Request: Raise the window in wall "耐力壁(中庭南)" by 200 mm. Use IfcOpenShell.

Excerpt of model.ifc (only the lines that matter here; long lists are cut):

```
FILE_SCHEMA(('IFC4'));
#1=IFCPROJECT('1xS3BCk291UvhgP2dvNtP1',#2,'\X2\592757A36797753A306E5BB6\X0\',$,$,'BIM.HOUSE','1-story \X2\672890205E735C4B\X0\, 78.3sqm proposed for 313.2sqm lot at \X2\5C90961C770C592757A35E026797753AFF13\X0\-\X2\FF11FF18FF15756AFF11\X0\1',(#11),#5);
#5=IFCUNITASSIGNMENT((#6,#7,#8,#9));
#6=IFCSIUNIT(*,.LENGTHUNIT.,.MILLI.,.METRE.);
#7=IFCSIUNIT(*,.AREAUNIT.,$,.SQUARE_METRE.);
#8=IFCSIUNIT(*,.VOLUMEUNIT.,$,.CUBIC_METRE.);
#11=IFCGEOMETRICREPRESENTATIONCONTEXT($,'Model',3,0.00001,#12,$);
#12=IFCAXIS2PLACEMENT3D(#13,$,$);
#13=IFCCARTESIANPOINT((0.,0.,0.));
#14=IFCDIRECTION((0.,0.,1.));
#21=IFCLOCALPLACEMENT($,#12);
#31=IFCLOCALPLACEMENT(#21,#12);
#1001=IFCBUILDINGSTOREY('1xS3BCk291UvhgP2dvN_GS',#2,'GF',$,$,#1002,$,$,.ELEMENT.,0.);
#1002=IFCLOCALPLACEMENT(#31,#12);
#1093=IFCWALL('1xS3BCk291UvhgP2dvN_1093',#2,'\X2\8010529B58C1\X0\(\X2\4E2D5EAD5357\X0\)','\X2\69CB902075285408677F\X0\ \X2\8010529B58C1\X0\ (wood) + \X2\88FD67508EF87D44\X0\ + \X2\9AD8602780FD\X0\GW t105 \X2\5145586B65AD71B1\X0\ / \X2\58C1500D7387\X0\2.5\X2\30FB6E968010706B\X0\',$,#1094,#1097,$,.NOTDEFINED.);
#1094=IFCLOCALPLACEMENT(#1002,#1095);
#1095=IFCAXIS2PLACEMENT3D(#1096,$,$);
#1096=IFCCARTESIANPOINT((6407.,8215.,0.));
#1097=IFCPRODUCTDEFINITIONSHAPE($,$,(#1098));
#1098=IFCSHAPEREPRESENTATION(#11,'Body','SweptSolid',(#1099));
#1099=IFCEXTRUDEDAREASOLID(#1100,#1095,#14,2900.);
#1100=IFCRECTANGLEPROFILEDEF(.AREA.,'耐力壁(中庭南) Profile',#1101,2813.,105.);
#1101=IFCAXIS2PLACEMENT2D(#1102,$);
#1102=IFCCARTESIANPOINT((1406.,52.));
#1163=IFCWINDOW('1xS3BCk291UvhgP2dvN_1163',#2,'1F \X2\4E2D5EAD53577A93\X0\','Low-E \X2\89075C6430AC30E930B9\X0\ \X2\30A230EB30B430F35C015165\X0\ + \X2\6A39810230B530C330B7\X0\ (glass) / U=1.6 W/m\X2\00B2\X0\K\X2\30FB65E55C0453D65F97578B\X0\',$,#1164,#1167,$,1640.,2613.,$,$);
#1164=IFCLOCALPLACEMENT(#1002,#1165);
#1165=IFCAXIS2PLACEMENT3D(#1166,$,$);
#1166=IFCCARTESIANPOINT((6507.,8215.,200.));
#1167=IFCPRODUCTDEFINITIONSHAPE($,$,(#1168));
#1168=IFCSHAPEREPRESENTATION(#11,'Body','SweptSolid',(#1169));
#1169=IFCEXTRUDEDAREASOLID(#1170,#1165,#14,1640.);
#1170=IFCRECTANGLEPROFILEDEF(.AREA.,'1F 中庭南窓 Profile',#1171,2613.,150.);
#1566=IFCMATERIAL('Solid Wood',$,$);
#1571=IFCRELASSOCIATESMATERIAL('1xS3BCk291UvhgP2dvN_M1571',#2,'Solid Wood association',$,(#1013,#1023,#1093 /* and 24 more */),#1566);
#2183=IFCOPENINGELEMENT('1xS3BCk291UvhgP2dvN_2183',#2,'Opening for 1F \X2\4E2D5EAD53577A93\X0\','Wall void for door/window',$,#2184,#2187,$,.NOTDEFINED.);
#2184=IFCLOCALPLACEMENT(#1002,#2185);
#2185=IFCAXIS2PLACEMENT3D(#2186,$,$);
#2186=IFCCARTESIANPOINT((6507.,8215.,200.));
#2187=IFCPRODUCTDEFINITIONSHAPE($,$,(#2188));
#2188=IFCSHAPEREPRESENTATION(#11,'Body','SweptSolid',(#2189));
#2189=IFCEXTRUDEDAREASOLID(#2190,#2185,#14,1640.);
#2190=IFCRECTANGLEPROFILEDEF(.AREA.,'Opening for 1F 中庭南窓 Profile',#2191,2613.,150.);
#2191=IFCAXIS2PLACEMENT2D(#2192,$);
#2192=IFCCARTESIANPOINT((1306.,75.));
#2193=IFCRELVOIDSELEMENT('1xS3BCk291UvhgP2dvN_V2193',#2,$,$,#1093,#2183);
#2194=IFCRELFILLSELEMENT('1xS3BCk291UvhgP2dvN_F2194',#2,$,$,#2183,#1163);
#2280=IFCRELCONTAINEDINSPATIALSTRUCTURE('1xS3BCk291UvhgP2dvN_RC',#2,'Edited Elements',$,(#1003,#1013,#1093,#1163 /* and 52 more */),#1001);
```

```python
import numpy as np
import ifcopenshell
import ifcopenshell.api.geometry
import ifcopenshell.util.placement
import ifcopenshell.util.unit

model = ifcopenshell.open("model.ifc")
unit_scale = ifcopenshell.util.unit.calculate_unit_scale(model)

window = model.by_guid("1xS3BCk291UvhgP2dvN_1163")
opening = window.FillsVoids[0].RelatingOpeningElement
dz = 0.2 / unit_scale

shift = np.array([0.0, 0.0, dz])
# The window is not placed relative to its opening, so move both.
for product in (opening, window):
    matrix = ifcopenshell.util.placement.get_local_placement(product.ObjectPlacement)
    matrix[:3, 3] += shift
    ifcopenshell.api.geometry.edit_object_placement(model, product=product, matrix=matrix, is_si=False)

print(f"moved by {dz * unit_scale:+.3f} m")

model.write("model-out.ifc")
```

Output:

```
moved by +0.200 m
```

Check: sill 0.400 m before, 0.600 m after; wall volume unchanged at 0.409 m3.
